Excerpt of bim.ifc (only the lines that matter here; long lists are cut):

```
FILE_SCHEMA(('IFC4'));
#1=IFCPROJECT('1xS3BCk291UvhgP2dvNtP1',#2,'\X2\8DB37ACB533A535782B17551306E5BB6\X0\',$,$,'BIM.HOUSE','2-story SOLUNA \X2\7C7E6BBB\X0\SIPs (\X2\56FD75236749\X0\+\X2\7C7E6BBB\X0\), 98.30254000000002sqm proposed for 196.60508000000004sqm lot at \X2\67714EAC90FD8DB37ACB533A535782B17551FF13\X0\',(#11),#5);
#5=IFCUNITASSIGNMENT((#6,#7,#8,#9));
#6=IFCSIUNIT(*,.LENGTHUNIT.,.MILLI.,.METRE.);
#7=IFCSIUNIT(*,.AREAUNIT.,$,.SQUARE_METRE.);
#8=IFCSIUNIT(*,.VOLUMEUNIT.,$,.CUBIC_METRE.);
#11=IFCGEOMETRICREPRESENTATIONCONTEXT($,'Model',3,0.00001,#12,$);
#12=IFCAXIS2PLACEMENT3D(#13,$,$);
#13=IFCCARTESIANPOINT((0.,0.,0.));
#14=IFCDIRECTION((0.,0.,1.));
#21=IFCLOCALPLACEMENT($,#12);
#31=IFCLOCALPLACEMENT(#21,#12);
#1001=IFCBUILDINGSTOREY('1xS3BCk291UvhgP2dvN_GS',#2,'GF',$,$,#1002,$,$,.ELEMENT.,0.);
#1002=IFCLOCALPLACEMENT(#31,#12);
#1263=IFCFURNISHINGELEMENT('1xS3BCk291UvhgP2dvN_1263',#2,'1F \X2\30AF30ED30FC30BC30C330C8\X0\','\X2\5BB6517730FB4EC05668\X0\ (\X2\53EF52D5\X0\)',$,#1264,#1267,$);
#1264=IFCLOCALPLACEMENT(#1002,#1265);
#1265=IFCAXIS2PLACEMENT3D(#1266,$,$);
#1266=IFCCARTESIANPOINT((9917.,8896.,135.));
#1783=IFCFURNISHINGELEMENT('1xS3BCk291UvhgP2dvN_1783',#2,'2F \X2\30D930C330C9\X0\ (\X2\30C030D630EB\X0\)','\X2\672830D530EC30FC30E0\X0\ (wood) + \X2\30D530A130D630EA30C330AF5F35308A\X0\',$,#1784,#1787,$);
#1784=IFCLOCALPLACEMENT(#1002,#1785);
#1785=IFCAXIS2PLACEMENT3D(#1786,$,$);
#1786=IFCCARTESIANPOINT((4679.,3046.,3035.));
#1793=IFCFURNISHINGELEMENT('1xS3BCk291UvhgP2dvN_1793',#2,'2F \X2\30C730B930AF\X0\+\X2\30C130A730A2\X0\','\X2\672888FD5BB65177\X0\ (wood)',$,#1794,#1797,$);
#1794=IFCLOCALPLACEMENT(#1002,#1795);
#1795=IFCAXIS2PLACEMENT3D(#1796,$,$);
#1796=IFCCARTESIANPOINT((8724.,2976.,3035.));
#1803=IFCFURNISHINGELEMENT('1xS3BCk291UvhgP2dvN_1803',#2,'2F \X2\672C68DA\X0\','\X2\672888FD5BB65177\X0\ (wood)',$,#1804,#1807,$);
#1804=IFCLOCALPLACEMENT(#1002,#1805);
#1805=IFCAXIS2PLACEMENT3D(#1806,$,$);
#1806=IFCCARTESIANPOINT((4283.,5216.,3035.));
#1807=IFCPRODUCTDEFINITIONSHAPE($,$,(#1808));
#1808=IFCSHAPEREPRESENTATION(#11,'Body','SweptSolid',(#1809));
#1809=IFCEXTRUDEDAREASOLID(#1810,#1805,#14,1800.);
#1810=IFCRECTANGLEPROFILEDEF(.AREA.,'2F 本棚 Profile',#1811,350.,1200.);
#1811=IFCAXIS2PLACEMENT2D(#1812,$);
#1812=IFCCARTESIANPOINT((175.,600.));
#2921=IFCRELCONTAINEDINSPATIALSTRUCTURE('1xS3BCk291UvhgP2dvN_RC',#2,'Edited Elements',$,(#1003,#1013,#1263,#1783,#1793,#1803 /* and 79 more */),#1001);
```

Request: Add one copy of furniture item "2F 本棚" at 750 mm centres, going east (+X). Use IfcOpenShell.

```python
import numpy as np
import ifcopenshell
import ifcopenshell.api.geometry
import ifcopenshell.api.root
import ifcopenshell.util.element
import ifcopenshell.util.placement
import ifcopenshell.util.unit

model = ifcopenshell.open("bim.ifc")
unit_scale = ifcopenshell.util.unit.calculate_unit_scale(model)


def reuse_history(source, copy):
    """copy_class also copies each property set's owner history, people and application; keep the originals."""
    for rel in copy.IsDefinedBy:
        if rel.is_a("IfcRelDefinesByProperties") and (history := rel.RelatingPropertyDefinition.OwnerHistory):
            rel.RelatingPropertyDefinition.OwnerHistory = source.OwnerHistory
            ifcopenshell.util.element.remove_deep2(model, history)


source = model.by_guid("1xS3BCk291UvhgP2dvN_1803")
base = ifcopenshell.util.placement.get_local_placement(source.ObjectPlacement)
step = np.array([1.0, 0.0, 0.0]) * 0.75 / unit_scale

for i in range(1, 2):
    copy = ifcopenshell.api.root.copy_class(model, product=source)
    copy.Representation = ifcopenshell.util.element.copy_deep(
        model, source.Representation, exclude=["IfcGeometricRepresentationContext", "IfcRepresentationMap"]
    )
    reuse_history(source, copy)
    matrix = base.copy()
    matrix[:3, 3] += i * step
    print("added at", matrix[:3, 3].round(3) + 0.0)
    ifcopenshell.api.geometry.edit_object_placement(model, product=copy, matrix=matrix, is_si=False)

model.write("bim_rev.ifc")
```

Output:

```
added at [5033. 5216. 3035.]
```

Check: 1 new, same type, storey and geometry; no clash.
